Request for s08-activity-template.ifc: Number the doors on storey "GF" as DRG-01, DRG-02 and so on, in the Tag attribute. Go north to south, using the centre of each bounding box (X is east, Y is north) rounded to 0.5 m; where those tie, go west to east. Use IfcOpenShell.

First a look at what the model holds.

```python
import ifcopenshell
import ifcopenshell.util.element
import ifcopenshell.util.placement

model = ifcopenshell.open("s08-activity-template.ifc")
print(model.schema)
storey = next(s for s in model.by_type("IfcBuildingStorey") if s.Name == "GF")
doors = [e for e in ifcopenshell.util.element.get_decomposition(storey) if e.is_a("IfcDoor")]
for e in sorted(doors, key=lambda e: e.id()):
    origin = ifcopenshell.util.placement.get_local_placement(e.ObjectPlacement)[:3, 3]
    print(e.id(), e.Tag, e.Name, origin.round(2) + 0.0, sep=" | ")
```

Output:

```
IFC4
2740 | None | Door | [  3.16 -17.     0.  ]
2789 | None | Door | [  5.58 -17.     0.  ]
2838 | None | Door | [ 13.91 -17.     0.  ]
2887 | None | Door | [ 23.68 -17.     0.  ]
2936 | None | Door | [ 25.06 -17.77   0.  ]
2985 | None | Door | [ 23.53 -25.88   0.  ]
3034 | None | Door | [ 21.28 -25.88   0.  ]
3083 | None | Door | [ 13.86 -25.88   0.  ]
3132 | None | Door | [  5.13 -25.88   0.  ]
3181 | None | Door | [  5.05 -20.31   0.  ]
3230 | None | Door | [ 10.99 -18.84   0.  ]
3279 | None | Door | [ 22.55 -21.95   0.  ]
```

```python
import ifcopenshell
import ifcopenshell.geom
import ifcopenshell.util.element
import ifcopenshell.util.shape

model = ifcopenshell.open("s08-activity-template.ifc")
settings = ifcopenshell.geom.settings()
settings.set("use-world-coords", True)


def centre(element):
    shape = ifcopenshell.geom.create_shape(settings, element)
    return ifcopenshell.util.shape.get_bbox_centroid(shape.geometry)


storey = next(s for s in model.by_type("IfcBuildingStorey") if s.Name == "GF")
doors = [e for e in ifcopenshell.util.element.get_decomposition(storey) if e.is_a("IfcDoor")]

# Insertion points can sit at a corner or the storey origin, so sort by the geometry (in metres).
centres = {e: centre(e) for e in doors}
doors.sort(key=lambda e: (-round(centres[e][1] / 0.5), centres[e][0]))

for i, e in enumerate(doors, start=1):
    number = f"DRG-{i:02d}"
    e.Tag = number
    print(e.id(), number)

model.write("s08-activity-template_updated.ifc")
```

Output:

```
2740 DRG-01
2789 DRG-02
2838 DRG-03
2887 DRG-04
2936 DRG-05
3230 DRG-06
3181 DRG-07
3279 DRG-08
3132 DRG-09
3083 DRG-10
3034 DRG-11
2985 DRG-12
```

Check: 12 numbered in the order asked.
